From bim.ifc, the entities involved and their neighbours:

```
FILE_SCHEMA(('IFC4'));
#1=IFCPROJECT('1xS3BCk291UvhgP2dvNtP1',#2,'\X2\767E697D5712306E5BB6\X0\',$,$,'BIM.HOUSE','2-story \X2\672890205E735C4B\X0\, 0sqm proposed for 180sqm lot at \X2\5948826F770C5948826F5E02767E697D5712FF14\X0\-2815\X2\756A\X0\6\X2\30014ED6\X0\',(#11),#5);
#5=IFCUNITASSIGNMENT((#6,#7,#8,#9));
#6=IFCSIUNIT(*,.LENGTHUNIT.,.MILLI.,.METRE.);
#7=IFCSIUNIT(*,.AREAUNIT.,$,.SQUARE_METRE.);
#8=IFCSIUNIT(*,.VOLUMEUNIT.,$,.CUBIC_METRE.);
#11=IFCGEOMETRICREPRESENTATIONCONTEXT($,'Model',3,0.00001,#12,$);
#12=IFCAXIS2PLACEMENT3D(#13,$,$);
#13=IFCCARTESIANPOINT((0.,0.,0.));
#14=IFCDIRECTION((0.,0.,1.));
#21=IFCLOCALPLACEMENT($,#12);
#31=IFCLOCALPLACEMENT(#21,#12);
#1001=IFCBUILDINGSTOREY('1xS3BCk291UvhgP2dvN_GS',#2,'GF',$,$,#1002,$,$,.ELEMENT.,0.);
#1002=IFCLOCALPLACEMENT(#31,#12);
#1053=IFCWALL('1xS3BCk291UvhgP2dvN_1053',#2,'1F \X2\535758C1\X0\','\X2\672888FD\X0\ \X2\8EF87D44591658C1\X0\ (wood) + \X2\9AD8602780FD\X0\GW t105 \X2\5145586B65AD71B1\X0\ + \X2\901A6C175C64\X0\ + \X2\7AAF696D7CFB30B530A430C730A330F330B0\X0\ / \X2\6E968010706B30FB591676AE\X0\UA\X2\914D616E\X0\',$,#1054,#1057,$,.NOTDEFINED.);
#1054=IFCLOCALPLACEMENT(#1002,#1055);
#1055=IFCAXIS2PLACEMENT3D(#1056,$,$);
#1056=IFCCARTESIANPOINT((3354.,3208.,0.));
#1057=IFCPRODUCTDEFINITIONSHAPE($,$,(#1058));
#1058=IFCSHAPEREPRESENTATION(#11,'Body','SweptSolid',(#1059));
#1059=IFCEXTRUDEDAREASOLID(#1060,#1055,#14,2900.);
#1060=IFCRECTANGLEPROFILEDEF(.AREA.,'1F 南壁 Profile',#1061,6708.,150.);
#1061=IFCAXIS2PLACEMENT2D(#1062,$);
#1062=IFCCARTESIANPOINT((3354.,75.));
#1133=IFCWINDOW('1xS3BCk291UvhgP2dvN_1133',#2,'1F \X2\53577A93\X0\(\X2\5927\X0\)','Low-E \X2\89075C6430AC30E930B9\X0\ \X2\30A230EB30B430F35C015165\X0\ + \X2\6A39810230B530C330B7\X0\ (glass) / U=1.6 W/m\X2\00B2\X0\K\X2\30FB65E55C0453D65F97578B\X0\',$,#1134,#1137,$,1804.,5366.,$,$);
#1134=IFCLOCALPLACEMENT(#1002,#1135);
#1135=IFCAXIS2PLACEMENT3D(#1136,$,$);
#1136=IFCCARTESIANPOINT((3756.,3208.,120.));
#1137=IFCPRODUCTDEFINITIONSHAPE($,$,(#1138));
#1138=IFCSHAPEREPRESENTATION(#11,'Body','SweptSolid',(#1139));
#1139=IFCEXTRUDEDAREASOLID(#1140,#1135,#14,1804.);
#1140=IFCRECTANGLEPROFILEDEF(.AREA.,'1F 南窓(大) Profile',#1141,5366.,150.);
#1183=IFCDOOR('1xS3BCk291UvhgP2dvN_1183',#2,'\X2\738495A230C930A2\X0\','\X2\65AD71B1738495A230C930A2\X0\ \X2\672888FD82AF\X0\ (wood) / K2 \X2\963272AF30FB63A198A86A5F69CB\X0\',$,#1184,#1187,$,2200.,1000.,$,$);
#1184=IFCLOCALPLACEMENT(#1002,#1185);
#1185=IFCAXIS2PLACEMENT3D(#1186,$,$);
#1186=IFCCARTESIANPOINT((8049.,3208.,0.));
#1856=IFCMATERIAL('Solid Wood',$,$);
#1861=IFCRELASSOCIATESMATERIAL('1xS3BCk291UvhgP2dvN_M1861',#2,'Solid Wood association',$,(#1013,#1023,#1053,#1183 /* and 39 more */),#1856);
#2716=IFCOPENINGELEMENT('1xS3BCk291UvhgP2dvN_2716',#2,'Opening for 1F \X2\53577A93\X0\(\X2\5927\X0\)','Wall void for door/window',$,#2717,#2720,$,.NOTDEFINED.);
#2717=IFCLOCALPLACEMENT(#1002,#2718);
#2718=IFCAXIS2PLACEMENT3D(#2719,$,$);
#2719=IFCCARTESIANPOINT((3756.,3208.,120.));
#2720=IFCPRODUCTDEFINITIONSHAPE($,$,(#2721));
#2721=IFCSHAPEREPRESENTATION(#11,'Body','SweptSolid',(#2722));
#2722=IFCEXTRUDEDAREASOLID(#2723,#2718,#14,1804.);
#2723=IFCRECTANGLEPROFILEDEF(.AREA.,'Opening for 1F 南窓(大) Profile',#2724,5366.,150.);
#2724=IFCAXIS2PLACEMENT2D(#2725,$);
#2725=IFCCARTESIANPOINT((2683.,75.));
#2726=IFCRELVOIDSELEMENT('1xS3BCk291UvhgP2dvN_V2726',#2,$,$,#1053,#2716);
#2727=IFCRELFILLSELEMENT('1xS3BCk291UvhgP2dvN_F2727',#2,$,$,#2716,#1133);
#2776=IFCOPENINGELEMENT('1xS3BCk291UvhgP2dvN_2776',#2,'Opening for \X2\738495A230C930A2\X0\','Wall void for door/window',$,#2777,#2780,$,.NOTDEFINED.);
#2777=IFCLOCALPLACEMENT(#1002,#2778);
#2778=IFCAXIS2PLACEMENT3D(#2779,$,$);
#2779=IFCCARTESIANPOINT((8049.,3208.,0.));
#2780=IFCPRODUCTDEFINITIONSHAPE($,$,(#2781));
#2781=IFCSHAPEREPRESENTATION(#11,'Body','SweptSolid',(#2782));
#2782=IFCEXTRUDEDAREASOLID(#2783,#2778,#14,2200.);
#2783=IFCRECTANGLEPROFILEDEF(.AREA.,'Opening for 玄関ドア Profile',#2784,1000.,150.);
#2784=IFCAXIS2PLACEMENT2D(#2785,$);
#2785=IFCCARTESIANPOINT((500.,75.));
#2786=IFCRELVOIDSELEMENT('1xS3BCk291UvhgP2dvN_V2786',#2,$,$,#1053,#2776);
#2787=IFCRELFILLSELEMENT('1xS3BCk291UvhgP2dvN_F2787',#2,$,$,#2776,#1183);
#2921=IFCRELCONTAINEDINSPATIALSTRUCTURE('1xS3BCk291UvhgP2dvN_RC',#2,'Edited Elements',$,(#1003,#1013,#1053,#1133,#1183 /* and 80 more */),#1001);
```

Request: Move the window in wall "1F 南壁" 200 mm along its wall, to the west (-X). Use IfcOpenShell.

```python
import ifcopenshell
import ifcopenshell.api.geometry
import ifcopenshell.util.placement
import ifcopenshell.util.unit

model = ifcopenshell.open("bim.ifc")
unit_scale = ifcopenshell.util.unit.calculate_unit_scale(model)

window = model.by_id(1133)
opening = window.FillsVoids[0].RelatingOpeningElement
wall = opening.VoidsElements[0].RelatingBuildingElement

wall_matrix = ifcopenshell.util.placement.get_local_placement(wall.ObjectPlacement)
shift = wall_matrix[:3, 0] * -0.2 / unit_scale
before = ifcopenshell.util.placement.get_local_placement(window.ObjectPlacement)[:3, 3].copy()

# The window is not placed relative to its opening, so move both.
for product in (opening, window):
    matrix = ifcopenshell.util.placement.get_local_placement(product.ObjectPlacement)
    matrix[:3, 3] += shift
    ifcopenshell.api.geometry.edit_object_placement(model, product=product, matrix=matrix, is_si=False)

after = ifcopenshell.util.placement.get_local_placement(window.ObjectPlacement)[:3, 3]
print("window moved by", (after - before).round(3) + 0.0)

model.write("bim-out.ifc")
```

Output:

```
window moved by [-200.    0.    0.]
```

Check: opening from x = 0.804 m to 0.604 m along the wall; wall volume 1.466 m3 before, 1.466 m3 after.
